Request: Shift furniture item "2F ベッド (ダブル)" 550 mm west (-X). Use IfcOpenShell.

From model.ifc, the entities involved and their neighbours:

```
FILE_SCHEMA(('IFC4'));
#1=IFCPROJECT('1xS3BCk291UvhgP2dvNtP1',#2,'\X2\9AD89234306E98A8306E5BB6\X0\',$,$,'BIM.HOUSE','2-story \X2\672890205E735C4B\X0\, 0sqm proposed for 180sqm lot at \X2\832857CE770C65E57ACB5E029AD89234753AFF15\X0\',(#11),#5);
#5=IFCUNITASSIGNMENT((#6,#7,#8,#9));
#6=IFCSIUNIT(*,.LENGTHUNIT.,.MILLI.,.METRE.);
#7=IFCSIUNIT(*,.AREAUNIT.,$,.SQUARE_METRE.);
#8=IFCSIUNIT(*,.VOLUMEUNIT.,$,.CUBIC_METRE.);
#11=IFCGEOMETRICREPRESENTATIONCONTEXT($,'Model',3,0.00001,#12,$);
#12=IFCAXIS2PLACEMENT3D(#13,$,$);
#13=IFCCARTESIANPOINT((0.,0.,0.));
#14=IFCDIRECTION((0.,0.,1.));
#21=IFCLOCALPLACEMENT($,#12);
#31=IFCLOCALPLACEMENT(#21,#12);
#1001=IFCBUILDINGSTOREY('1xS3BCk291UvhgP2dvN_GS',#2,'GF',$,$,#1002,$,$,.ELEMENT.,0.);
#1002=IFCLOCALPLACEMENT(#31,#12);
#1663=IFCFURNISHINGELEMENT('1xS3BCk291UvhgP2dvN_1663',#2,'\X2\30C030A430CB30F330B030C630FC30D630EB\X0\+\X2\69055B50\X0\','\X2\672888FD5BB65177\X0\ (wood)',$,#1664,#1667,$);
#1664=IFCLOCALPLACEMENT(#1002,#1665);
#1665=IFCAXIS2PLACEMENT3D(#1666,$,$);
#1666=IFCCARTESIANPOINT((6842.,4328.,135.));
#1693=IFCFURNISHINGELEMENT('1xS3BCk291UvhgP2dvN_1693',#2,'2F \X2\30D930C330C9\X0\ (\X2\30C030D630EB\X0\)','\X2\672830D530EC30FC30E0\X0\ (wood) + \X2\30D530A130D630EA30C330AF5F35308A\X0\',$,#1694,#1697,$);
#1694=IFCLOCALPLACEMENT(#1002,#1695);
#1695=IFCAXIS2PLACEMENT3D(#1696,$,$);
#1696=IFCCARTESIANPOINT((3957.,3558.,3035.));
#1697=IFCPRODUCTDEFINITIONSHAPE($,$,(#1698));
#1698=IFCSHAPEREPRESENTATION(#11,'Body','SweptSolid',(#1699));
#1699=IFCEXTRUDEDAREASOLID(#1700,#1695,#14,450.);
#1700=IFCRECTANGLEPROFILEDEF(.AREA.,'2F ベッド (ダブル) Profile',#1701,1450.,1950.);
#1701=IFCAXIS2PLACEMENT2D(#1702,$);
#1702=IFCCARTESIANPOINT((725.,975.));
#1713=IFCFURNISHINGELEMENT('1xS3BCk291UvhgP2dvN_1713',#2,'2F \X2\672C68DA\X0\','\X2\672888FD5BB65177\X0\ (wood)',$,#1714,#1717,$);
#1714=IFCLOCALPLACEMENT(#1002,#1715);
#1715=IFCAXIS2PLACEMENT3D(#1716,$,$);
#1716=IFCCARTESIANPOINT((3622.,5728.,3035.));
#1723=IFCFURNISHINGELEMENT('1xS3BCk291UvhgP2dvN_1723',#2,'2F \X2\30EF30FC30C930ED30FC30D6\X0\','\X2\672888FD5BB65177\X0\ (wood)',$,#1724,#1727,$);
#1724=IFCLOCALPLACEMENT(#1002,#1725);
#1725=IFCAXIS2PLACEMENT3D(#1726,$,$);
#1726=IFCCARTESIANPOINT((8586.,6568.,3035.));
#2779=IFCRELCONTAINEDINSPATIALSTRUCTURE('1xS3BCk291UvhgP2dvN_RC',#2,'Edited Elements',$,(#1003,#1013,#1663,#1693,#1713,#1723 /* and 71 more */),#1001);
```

```python
import ifcopenshell
import ifcopenshell.api.geometry
import ifcopenshell.util.placement
import ifcopenshell.util.unit

model = ifcopenshell.open("model.ifc")
unit_scale = ifcopenshell.util.unit.calculate_unit_scale(model)

item = model.by_guid("1xS3BCk291UvhgP2dvN_1693")
matrix = ifcopenshell.util.placement.get_local_placement(item.ObjectPlacement)
matrix[0, 3] -= 0.55 / unit_scale
ifcopenshell.api.geometry.edit_object_placement(model, product=item, matrix=matrix, is_si=False)

print(ifcopenshell.util.placement.get_local_placement(item.ObjectPlacement).round(3) + 0.0)

model.write("model-out.ifc")
```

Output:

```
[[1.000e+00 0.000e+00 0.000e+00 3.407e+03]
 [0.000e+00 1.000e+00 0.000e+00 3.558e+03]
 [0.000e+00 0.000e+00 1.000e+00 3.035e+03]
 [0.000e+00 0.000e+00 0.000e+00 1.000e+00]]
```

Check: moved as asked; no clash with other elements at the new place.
